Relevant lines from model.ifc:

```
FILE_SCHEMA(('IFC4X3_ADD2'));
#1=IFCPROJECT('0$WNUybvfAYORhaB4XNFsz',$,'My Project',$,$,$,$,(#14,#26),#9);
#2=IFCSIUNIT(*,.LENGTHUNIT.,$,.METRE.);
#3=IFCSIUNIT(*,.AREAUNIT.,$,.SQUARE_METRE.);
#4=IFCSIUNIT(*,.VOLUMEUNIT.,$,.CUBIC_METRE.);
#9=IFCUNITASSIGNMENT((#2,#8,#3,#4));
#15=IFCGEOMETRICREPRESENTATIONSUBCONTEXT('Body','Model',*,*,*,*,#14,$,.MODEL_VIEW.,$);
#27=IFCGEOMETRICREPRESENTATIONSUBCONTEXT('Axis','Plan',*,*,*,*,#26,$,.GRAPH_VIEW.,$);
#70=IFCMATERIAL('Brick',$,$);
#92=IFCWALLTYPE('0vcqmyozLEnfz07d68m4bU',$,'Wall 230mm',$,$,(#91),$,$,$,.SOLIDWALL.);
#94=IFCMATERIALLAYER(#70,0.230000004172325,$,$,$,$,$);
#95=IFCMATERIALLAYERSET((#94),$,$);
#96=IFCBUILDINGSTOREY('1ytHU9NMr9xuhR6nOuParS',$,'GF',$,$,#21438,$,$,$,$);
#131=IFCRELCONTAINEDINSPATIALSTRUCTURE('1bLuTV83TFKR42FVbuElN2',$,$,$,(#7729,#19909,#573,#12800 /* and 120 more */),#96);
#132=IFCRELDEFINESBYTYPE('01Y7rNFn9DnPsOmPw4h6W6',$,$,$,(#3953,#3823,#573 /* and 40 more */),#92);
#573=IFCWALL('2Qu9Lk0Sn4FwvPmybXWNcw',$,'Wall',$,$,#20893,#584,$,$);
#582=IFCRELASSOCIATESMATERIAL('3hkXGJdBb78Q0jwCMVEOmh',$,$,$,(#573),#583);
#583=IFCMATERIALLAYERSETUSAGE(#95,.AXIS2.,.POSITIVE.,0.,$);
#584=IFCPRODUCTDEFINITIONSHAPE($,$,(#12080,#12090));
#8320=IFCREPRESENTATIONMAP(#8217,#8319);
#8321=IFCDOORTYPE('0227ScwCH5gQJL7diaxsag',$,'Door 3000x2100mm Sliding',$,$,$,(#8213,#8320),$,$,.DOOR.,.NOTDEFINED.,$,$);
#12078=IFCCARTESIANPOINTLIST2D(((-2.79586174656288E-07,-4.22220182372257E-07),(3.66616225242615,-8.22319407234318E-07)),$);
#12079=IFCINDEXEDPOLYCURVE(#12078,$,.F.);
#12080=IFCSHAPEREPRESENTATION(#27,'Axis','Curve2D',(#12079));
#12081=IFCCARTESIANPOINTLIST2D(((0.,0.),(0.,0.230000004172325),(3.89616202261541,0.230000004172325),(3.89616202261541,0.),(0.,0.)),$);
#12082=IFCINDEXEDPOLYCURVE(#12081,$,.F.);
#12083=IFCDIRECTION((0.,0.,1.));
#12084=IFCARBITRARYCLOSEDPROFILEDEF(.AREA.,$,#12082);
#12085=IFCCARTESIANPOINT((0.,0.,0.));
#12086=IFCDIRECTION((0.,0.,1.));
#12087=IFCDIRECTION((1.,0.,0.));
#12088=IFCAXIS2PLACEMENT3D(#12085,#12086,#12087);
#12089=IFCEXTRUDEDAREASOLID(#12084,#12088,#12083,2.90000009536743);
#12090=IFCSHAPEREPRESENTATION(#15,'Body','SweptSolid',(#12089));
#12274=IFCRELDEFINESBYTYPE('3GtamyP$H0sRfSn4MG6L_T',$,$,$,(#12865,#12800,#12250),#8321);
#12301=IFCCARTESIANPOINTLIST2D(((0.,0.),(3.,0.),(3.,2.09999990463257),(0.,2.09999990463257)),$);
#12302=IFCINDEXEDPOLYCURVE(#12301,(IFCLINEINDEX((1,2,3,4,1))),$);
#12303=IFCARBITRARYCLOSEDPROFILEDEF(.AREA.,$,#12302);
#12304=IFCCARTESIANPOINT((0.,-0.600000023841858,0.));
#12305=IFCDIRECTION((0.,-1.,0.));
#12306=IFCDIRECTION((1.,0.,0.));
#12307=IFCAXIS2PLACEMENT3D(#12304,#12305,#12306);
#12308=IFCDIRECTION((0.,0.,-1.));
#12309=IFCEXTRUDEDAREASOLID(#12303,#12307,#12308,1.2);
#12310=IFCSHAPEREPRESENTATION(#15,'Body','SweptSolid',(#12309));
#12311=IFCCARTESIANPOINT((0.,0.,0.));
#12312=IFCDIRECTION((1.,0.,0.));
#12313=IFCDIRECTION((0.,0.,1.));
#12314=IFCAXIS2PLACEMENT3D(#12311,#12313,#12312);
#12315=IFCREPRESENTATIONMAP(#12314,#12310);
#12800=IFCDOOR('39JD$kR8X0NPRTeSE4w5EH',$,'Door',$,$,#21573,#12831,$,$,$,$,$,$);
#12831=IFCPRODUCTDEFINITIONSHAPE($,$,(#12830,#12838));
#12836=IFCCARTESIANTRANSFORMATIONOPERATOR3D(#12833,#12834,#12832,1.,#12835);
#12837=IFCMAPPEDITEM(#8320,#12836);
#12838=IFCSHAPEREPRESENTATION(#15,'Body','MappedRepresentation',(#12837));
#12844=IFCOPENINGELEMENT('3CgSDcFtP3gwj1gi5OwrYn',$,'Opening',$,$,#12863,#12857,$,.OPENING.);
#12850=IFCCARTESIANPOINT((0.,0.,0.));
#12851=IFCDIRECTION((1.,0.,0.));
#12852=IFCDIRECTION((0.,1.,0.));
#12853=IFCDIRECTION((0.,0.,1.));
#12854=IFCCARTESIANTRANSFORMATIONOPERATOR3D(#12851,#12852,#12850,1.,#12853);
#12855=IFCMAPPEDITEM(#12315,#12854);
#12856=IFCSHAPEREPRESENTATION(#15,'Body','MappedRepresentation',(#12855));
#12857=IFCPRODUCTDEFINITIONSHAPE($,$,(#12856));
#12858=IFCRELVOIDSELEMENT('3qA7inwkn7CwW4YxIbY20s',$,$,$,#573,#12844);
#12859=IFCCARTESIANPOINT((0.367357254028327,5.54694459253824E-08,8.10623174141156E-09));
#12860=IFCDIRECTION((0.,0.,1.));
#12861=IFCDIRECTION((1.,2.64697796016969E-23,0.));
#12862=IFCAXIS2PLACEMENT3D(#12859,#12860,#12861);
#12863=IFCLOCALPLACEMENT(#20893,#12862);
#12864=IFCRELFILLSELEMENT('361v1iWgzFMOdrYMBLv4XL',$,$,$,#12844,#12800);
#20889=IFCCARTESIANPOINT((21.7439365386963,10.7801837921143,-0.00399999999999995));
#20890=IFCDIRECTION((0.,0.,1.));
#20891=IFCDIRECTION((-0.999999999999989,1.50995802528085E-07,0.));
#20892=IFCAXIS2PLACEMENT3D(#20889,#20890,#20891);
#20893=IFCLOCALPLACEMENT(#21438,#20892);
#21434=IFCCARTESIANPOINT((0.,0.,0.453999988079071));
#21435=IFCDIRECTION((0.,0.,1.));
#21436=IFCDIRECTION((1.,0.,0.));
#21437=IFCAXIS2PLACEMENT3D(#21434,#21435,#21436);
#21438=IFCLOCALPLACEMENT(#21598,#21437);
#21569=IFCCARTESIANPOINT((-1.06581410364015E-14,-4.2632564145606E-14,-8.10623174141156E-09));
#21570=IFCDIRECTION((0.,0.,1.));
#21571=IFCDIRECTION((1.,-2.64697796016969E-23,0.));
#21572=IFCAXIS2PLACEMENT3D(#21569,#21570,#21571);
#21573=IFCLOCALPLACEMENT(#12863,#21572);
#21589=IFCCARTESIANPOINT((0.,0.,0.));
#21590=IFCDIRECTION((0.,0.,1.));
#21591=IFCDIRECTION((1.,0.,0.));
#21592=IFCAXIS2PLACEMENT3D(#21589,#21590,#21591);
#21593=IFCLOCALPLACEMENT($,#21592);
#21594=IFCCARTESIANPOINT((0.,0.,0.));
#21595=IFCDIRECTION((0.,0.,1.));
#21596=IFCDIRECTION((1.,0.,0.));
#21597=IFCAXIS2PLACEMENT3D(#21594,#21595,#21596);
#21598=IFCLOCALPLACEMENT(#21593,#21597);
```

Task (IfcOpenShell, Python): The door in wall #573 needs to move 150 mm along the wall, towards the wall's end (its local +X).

```python
import ifcopenshell
import ifcopenshell.api.geometry
import ifcopenshell.util.placement

model = ifcopenshell.open("model.ifc")

door = model.by_guid("39JD$kR8X0NPRTeSE4w5EH")
opening = door.FillsVoids[0].RelatingOpeningElement
wall = opening.VoidsElements[0].RelatingBuildingElement

wall_matrix = ifcopenshell.util.placement.get_local_placement(wall.ObjectPlacement)
shift = wall_matrix[:3, 0] * 0.15
before = ifcopenshell.util.placement.get_local_placement(door.ObjectPlacement)[:3, 3].copy()

# The door is placed relative to its opening, so it follows when the opening moves.
matrix = ifcopenshell.util.placement.get_local_placement(opening.ObjectPlacement)
matrix[:3, 3] += shift
ifcopenshell.api.geometry.edit_object_placement(
    model, product=opening, matrix=matrix, is_si=False, should_transform_children=True
)

after = ifcopenshell.util.placement.get_local_placement(door.ObjectPlacement)[:3, 3]
print("door moved by", (after - before).round(3) + 0.0)

model.write("model_updated.ifc")
```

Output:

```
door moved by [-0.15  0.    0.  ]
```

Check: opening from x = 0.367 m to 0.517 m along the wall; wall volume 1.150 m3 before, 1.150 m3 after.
